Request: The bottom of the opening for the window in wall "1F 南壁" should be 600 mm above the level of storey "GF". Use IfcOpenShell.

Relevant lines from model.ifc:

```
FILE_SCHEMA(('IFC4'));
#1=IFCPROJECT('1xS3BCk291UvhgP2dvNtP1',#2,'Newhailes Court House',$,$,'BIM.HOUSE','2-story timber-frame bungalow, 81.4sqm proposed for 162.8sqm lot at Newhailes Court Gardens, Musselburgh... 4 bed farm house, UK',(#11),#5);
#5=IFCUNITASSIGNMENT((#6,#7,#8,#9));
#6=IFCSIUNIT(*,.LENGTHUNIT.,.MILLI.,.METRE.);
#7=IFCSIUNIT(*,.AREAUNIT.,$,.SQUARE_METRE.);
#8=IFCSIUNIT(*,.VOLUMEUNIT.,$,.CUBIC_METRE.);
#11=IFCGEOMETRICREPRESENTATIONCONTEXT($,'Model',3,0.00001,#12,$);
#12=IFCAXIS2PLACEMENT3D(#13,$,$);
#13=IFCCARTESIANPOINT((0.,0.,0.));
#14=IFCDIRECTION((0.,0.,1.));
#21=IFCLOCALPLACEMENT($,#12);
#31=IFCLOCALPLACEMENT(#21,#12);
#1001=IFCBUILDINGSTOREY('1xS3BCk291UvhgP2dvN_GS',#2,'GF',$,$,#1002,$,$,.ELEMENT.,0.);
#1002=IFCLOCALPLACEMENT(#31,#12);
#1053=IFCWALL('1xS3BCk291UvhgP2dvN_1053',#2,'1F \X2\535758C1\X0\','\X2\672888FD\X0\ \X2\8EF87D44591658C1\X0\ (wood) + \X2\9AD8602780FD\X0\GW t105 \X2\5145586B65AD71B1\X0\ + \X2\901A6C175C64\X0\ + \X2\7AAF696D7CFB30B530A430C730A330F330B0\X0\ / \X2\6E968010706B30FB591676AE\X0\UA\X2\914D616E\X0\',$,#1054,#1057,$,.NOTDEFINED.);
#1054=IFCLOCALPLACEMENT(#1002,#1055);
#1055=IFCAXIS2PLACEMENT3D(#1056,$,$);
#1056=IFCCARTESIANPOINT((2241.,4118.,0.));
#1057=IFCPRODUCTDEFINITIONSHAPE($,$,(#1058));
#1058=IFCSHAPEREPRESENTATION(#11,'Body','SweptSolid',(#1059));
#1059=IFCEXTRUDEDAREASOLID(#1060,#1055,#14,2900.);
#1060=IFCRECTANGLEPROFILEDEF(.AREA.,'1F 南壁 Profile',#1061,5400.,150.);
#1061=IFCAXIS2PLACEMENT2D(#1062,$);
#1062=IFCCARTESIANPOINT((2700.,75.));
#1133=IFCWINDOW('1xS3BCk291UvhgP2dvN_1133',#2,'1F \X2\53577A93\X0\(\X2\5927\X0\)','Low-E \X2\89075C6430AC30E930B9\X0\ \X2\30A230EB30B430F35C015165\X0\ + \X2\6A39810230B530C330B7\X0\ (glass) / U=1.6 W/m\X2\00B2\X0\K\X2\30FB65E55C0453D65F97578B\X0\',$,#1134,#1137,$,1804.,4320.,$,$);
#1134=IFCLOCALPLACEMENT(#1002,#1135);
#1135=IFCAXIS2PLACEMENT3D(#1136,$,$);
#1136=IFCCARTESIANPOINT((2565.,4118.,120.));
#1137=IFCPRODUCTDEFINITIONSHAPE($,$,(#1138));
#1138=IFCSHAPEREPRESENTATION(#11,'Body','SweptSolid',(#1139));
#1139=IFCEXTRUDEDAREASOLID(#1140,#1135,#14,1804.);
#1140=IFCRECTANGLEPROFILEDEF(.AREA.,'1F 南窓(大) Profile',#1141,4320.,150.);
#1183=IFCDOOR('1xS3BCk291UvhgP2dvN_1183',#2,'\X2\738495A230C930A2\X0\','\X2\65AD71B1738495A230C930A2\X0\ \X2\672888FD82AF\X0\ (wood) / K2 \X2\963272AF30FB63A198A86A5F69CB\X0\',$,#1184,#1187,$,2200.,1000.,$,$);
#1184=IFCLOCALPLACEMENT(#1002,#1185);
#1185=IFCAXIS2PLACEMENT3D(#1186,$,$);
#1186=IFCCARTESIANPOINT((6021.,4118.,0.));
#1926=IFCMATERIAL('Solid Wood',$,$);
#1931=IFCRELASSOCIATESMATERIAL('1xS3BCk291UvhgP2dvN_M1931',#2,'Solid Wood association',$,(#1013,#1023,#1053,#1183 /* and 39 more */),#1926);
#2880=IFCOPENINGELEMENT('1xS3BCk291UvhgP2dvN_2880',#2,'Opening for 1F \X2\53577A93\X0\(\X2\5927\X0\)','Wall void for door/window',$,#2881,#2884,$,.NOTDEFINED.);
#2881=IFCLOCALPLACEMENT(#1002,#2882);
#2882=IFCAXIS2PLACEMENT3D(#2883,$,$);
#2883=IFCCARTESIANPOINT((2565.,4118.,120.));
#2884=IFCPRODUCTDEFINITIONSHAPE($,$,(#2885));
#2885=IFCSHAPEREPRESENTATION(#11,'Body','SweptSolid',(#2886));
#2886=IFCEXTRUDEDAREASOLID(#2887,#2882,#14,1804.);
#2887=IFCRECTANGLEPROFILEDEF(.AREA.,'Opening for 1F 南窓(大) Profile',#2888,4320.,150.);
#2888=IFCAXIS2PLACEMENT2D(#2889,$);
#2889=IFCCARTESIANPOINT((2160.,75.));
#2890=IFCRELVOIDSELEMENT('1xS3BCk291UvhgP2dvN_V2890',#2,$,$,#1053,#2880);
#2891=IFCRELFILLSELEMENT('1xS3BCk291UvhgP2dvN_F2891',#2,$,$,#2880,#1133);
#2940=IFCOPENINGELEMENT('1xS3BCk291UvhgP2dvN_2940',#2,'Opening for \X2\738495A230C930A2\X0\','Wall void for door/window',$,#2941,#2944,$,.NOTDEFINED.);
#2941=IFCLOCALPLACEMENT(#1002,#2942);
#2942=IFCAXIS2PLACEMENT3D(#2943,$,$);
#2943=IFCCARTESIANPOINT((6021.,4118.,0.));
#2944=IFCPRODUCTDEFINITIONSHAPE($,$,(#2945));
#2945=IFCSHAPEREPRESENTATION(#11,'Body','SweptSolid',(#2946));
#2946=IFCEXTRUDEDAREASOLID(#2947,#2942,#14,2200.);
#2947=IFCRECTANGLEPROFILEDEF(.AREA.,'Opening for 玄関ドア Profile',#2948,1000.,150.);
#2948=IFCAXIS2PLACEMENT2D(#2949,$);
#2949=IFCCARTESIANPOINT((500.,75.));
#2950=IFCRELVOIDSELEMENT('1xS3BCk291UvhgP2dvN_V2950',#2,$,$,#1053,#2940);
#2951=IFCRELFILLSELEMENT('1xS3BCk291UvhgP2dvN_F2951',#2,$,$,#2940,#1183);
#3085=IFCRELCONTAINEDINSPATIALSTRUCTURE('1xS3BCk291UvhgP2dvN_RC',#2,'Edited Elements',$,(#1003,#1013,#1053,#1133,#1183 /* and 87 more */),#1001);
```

```python
import numpy as np
import ifcopenshell
import ifcopenshell.api.geometry
import ifcopenshell.geom
import ifcopenshell.util.element
import ifcopenshell.util.placement
import ifcopenshell.util.shape
import ifcopenshell.util.unit

model = ifcopenshell.open("model.ifc")
unit_scale = ifcopenshell.util.unit.calculate_unit_scale(model)

window = model.by_guid("1xS3BCk291UvhgP2dvN_1133")
opening = window.FillsVoids[0].RelatingOpeningElement
storey = ifcopenshell.util.element.get_container(window, ifc_class="IfcBuildingStorey")
level = ifcopenshell.util.placement.get_local_placement(storey.ObjectPlacement)[2, 3]

# The opening's origin need not be at the sill, so measure its lowest point.
shape = ifcopenshell.geom.create_shape(ifcopenshell.geom.settings(), opening)
bottom = ifcopenshell.util.shape.get_shape_bottom_elevation(shape, shape.geometry) / unit_scale
dz = level + 0.6 / unit_scale - bottom

shift = np.array([0.0, 0.0, dz])
# The window is not placed relative to its opening, so move both.
for product in (opening, window):
    matrix = ifcopenshell.util.placement.get_local_placement(product.ObjectPlacement)
    matrix[:3, 3] += shift
    ifcopenshell.api.geometry.edit_object_placement(model, product=product, matrix=matrix, is_si=False)

print(f"moved by {dz * unit_scale:+.3f} m")

model.write("model_v2.ifc")
```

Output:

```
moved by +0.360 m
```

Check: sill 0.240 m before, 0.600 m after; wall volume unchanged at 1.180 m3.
